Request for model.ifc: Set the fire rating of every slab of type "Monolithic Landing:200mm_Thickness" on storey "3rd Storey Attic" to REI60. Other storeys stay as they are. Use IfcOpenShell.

First a look at what the model holds.

```python
import ifcopenshell
import ifcopenshell.util.element

model = ifcopenshell.open("model.ifc")
print(model.schema)
storey = next(s for s in model.by_type("IfcBuildingStorey") if s.Name == "3rd Storey Attic")
slabs = [e for e in ifcopenshell.util.element.get_decomposition(storey) if e.is_a("IfcSlab")]
seen = {}
for e in slabs:
    element_type = ifcopenshell.util.element.get_type(e)
    key = (element_type.Name if element_type != e and element_type else None, ifcopenshell.util.element.get_pset(e, "Pset_SlabCommon", "FireRating"))
    seen[key] = seen.get(key, 0) + 1
for (name, value), count in sorted(seen.items(), key=str):
    print(count, "x", name, "|", value)
```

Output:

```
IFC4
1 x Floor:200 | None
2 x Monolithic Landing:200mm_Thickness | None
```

```python
import ifcopenshell
import ifcopenshell.api.pset
import ifcopenshell.util.element

model = ifcopenshell.open("model.ifc")

storey = next(s for s in model.by_type("IfcBuildingStorey") if s.Name == "3rd Storey Attic")
slabs = [e for e in ifcopenshell.util.element.get_decomposition(storey) if e.is_a("IfcSlab")]

count = 0
for e in slabs:
    element_type = ifcopenshell.util.element.get_type(e)
    if element_type in (None, e) or element_type.Name != "Monolithic Landing:200mm_Thickness":
        continue
    # add_pset returns the element's existing set when there is one.
    pset = ifcopenshell.api.pset.add_pset(model, product=e, name="Pset_SlabCommon")
    ifcopenshell.api.pset.edit_pset(model, pset=pset, properties={"FireRating": "REI60"})
    count += 1

print(count, "slabs updated")

model.write("model_edited.ifc")
```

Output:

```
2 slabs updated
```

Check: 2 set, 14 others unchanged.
